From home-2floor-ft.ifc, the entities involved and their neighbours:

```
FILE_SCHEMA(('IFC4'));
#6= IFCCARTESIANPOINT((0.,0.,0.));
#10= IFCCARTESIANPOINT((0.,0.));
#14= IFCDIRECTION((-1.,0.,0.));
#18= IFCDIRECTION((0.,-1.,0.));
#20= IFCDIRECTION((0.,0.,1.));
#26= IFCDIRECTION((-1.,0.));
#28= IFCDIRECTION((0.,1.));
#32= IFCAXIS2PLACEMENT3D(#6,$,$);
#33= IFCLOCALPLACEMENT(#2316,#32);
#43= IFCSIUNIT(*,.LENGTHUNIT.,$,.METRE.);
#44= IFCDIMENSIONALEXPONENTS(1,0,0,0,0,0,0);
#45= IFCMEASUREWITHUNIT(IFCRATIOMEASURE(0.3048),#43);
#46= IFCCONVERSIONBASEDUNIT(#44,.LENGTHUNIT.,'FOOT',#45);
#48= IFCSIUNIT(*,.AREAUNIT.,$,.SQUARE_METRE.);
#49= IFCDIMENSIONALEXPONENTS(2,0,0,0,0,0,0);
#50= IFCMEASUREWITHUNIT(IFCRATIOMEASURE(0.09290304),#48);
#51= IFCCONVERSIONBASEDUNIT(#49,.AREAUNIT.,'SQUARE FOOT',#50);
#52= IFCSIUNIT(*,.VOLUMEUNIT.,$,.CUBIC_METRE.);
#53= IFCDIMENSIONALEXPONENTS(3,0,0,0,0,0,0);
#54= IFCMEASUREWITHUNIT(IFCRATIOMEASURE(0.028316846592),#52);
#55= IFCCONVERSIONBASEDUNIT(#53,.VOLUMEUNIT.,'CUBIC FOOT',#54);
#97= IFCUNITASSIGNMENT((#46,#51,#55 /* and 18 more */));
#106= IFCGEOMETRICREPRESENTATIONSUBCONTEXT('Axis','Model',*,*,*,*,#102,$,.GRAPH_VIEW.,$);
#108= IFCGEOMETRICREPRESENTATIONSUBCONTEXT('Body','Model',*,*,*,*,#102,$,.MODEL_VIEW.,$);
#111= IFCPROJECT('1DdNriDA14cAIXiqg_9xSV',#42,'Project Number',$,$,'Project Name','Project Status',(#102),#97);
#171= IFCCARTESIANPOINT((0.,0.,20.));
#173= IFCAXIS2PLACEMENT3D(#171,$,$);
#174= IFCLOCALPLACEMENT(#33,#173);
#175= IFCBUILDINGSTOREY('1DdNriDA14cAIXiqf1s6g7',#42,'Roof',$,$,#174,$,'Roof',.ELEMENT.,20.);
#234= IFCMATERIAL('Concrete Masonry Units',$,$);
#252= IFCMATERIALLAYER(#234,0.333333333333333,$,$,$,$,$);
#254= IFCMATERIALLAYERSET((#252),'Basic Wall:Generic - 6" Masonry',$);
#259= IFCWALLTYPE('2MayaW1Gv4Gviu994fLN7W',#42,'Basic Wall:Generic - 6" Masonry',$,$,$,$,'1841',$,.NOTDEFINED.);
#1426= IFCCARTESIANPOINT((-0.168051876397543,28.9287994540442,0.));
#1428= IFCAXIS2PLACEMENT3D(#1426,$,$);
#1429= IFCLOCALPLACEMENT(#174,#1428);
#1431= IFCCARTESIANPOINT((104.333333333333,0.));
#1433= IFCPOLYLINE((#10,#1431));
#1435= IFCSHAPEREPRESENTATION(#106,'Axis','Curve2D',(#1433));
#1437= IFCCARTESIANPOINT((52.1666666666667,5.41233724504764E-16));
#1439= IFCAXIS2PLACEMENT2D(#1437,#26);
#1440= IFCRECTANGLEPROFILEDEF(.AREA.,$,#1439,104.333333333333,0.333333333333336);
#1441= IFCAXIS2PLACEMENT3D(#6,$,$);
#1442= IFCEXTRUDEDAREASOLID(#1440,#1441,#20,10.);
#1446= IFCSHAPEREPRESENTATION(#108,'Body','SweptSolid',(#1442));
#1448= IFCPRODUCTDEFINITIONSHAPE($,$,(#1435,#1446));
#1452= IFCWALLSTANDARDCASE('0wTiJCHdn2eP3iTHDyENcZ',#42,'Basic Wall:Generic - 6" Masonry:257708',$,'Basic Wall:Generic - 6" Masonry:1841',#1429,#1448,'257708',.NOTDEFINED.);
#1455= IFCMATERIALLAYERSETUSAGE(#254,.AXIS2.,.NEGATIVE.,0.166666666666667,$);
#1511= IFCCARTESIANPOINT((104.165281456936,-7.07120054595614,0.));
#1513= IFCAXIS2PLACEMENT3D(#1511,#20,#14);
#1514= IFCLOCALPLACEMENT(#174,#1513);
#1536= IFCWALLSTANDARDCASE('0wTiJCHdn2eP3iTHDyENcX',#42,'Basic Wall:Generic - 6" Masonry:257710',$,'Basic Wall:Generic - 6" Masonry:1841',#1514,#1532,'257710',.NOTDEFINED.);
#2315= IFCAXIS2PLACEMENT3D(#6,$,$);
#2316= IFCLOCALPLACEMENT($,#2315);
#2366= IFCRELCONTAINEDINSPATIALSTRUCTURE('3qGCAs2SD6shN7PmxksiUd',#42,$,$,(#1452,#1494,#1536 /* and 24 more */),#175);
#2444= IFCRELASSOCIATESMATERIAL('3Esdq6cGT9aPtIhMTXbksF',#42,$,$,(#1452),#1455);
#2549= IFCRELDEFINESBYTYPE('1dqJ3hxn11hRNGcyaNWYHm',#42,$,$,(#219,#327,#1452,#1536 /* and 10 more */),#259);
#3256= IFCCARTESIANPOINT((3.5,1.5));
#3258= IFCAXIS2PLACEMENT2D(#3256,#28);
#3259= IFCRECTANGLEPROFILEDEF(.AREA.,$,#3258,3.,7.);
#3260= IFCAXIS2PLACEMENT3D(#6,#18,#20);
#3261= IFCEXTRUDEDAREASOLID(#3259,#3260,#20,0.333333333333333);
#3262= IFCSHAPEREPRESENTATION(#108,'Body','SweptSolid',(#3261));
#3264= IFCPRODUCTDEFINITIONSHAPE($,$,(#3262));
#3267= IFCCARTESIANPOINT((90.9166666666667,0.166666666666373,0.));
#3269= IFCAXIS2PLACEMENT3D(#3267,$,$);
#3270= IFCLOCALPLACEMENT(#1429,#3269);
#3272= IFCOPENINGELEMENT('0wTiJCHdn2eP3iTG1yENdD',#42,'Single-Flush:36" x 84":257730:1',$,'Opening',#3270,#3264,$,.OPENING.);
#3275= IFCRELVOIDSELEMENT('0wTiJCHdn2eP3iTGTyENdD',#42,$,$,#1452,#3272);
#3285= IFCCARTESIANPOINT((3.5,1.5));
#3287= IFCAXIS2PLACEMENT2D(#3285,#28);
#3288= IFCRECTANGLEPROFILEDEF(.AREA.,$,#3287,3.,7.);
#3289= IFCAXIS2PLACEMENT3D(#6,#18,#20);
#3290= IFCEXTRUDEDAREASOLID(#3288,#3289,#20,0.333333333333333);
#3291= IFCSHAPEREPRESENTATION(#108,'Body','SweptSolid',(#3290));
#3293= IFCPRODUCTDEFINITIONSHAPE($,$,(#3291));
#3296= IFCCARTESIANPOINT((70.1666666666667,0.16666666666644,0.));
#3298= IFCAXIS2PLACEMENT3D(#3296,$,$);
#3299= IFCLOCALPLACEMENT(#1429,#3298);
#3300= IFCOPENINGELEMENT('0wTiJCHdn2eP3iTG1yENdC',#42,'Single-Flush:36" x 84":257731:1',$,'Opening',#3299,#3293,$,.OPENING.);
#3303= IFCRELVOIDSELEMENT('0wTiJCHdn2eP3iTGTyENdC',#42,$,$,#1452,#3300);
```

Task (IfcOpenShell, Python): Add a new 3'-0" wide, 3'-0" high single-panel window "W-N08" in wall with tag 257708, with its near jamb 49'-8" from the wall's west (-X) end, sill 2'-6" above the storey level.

```python
import numpy as np
import ifcopenshell
import ifcopenshell.api.feature
import ifcopenshell.api.geometry
import ifcopenshell.api.root
import ifcopenshell.api.spatial
import ifcopenshell.geom
import ifcopenshell.util.element
import ifcopenshell.util.placement
import ifcopenshell.util.representation
import ifcopenshell.util.shape
import ifcopenshell.util.unit

model = ifcopenshell.open("home-2floor-ft.ifc")
unit_scale = ifcopenshell.util.unit.calculate_unit_scale(model)
settings = ifcopenshell.geom.settings()


def volume(element):
    """Net volume in cubic metres, openings subtracted."""
    shape = ifcopenshell.geom.create_shape(settings, element)
    return ifcopenshell.util.shape.get_volume(shape.geometry)


wall = model.by_id(1452)
storey = ifcopenshell.util.element.get_container(wall, ifc_class="IfcBuildingStorey")
context = ifcopenshell.util.representation.get_context(model, "Model", "Body", "MODEL_VIEW")
before = volume(wall)

width, height, from_end, sill = 0.9144, 0.9144, 15.1384, 0.762  # metres

# The wall runs along its own X axis, and the end named is its -X end.
wall_shape = ifcopenshell.geom.create_shape(settings, wall)
x, y, z = ifcopenshell.util.shape.get_vertices(wall_shape.geometry).T
start = x.min() + from_end
face, thickness = float(y.min()), float(y.max() - y.min())
wall_matrix = ifcopenshell.util.placement.get_local_placement(wall.ObjectPlacement)
level = ifcopenshell.util.placement.get_local_placement(storey.ObjectPlacement)[2, 3]


def in_wall(x, y):
    """Placement at x, y metres in the wall's axes, at sill height."""
    matrix = wall_matrix.copy()
    matrix[:, 3] = wall_matrix @ np.array([x / unit_scale, y / unit_scale, 0.0, 1.0])
    matrix[2, 3] = level + sill / unit_scale
    return matrix


# Opening: a box that overshoots both wall faces by 50 mm.
opening = ifcopenshell.api.root.create_entity(model, ifc_class="IfcOpeningElement", predefined_type="OPENING")
box = ifcopenshell.api.geometry.add_wall_representation(
    model, context=context, length=width, height=height, thickness=thickness + 0.1
)
ifcopenshell.api.geometry.assign_representation(model, product=opening, representation=box)
ifcopenshell.api.geometry.edit_object_placement(model, product=opening, matrix=in_wall(start, face - 0.05), is_si=False)
ifcopenshell.api.feature.add_feature(model, feature=opening, element=wall)

window = ifcopenshell.api.root.create_entity(model, ifc_class="IfcWindow", name="W-N08", predefined_type="WINDOW")
window.OverallWidth, window.OverallHeight = width / unit_scale, height / unit_scale
window.PartitioningType = "SINGLE_PANEL"
body = ifcopenshell.api.geometry.add_window_representation(
    model,
    context=context,
    overall_width=window.OverallWidth,
    overall_height=window.OverallHeight,
    partition_type="SINGLE_PANEL",
)
ifcopenshell.api.geometry.assign_representation(model, product=window, representation=body)
ifcopenshell.api.spatial.assign_container(model, products=[window], relating_structure=storey)
ifcopenshell.api.feature.add_filling(model, opening=opening, element=window)

# Centre the window in the wall's thickness.
ifcopenshell.api.geometry.edit_object_placement(model, product=window, matrix=in_wall(start, face), is_si=False)
window_shape = ifcopenshell.geom.create_shape(settings, window)
depth = ifcopenshell.util.shape.get_vertices(window_shape.geometry)[:, 1]
offset = face + thickness / 2 - (depth.min() + depth.max()) / 2
ifcopenshell.api.geometry.edit_object_placement(model, product=window, matrix=in_wall(start, offset), is_si=False)

after = volume(wall)

print(f"wall volume {before:.3f} -> {after:.3f} m3")

model.write("home-2floor-ft_v2.ifc")
```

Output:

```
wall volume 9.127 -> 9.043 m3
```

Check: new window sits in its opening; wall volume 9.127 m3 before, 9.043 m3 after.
